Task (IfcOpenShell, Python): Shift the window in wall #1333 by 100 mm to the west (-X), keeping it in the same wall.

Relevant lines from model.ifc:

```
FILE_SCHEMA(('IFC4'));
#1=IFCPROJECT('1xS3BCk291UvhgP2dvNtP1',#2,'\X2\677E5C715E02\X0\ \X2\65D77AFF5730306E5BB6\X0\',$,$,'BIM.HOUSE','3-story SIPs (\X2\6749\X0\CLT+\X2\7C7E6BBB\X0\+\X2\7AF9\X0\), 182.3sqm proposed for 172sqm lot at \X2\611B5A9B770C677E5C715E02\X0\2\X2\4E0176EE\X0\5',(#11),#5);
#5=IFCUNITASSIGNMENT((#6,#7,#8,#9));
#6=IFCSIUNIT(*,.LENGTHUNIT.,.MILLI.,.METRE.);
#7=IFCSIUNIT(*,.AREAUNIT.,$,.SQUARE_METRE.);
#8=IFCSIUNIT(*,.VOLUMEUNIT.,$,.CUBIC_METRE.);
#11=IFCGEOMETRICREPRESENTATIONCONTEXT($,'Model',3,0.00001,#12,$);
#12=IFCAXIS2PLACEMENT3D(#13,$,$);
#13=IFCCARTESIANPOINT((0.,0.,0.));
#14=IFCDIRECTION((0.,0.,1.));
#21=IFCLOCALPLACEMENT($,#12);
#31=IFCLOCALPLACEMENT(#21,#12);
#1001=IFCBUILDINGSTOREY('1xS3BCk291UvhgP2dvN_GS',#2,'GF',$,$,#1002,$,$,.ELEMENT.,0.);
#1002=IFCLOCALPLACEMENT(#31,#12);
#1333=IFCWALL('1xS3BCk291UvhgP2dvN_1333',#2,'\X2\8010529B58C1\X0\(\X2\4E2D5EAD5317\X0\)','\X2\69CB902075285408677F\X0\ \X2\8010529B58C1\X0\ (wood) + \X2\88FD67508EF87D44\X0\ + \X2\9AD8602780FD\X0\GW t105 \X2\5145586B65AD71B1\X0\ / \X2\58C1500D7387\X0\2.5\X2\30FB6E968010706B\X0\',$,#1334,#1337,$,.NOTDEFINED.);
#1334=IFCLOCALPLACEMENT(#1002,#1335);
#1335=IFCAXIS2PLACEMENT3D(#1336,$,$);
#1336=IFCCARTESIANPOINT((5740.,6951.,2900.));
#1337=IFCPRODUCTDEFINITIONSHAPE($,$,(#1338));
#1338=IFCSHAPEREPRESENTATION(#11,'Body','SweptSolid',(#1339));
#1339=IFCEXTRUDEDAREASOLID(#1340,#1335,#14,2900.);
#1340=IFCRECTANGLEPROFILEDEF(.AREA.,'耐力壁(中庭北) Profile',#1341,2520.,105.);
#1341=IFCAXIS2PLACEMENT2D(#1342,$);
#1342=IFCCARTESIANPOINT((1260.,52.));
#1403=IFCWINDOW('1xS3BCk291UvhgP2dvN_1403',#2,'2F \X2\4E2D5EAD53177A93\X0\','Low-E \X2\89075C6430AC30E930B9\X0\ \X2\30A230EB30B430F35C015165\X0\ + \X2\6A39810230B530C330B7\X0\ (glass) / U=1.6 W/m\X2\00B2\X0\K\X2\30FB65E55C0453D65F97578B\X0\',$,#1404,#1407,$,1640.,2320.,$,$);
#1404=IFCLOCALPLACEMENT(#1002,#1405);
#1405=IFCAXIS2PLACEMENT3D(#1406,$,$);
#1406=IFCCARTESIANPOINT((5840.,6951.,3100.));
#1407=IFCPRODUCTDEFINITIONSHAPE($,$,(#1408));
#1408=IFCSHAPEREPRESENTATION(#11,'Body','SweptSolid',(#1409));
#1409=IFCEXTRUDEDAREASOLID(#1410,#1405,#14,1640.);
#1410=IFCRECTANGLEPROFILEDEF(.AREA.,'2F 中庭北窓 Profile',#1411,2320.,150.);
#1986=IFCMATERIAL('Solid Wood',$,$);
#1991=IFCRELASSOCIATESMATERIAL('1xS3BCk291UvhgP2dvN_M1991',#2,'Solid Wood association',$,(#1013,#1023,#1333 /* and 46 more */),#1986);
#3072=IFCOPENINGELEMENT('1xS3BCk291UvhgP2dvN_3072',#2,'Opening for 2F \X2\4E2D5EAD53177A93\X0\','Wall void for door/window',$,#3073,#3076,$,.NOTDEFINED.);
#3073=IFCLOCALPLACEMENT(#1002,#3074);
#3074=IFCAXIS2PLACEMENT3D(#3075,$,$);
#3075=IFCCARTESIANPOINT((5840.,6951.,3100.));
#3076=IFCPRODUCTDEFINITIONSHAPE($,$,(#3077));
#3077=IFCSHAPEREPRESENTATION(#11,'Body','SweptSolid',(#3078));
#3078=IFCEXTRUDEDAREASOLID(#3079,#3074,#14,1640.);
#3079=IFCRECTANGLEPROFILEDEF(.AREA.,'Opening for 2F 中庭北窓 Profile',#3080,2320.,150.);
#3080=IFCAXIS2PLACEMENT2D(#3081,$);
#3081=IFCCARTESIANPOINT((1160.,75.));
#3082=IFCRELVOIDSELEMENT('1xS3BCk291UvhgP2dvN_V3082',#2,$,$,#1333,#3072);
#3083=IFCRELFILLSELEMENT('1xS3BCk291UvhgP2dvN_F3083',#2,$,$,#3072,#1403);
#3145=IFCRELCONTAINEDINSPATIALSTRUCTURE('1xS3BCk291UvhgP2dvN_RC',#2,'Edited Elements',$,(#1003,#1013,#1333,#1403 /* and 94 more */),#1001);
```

```python
import ifcopenshell
import ifcopenshell.api.geometry
import ifcopenshell.util.placement
import ifcopenshell.util.unit

model = ifcopenshell.open("model.ifc")
unit_scale = ifcopenshell.util.unit.calculate_unit_scale(model)

window = model.by_guid("1xS3BCk291UvhgP2dvN_1403")
opening = window.FillsVoids[0].RelatingOpeningElement
wall = opening.VoidsElements[0].RelatingBuildingElement

wall_matrix = ifcopenshell.util.placement.get_local_placement(wall.ObjectPlacement)
shift = wall_matrix[:3, 0] * -0.1 / unit_scale
before = ifcopenshell.util.placement.get_local_placement(window.ObjectPlacement)[:3, 3].copy()

# The window is not placed relative to its opening, so move both.
for product in (opening, window):
    matrix = ifcopenshell.util.placement.get_local_placement(product.ObjectPlacement)
    matrix[:3, 3] += shift
    ifcopenshell.api.geometry.edit_object_placement(model, product=product, matrix=matrix, is_si=False)

after = ifcopenshell.util.placement.get_local_placement(window.ObjectPlacement)[:3, 3]
print("window moved by", (after - before).round(3) + 0.0)

model.write("model_rev.ifc")
```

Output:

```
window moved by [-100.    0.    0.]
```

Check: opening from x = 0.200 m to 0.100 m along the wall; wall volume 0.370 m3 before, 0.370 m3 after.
